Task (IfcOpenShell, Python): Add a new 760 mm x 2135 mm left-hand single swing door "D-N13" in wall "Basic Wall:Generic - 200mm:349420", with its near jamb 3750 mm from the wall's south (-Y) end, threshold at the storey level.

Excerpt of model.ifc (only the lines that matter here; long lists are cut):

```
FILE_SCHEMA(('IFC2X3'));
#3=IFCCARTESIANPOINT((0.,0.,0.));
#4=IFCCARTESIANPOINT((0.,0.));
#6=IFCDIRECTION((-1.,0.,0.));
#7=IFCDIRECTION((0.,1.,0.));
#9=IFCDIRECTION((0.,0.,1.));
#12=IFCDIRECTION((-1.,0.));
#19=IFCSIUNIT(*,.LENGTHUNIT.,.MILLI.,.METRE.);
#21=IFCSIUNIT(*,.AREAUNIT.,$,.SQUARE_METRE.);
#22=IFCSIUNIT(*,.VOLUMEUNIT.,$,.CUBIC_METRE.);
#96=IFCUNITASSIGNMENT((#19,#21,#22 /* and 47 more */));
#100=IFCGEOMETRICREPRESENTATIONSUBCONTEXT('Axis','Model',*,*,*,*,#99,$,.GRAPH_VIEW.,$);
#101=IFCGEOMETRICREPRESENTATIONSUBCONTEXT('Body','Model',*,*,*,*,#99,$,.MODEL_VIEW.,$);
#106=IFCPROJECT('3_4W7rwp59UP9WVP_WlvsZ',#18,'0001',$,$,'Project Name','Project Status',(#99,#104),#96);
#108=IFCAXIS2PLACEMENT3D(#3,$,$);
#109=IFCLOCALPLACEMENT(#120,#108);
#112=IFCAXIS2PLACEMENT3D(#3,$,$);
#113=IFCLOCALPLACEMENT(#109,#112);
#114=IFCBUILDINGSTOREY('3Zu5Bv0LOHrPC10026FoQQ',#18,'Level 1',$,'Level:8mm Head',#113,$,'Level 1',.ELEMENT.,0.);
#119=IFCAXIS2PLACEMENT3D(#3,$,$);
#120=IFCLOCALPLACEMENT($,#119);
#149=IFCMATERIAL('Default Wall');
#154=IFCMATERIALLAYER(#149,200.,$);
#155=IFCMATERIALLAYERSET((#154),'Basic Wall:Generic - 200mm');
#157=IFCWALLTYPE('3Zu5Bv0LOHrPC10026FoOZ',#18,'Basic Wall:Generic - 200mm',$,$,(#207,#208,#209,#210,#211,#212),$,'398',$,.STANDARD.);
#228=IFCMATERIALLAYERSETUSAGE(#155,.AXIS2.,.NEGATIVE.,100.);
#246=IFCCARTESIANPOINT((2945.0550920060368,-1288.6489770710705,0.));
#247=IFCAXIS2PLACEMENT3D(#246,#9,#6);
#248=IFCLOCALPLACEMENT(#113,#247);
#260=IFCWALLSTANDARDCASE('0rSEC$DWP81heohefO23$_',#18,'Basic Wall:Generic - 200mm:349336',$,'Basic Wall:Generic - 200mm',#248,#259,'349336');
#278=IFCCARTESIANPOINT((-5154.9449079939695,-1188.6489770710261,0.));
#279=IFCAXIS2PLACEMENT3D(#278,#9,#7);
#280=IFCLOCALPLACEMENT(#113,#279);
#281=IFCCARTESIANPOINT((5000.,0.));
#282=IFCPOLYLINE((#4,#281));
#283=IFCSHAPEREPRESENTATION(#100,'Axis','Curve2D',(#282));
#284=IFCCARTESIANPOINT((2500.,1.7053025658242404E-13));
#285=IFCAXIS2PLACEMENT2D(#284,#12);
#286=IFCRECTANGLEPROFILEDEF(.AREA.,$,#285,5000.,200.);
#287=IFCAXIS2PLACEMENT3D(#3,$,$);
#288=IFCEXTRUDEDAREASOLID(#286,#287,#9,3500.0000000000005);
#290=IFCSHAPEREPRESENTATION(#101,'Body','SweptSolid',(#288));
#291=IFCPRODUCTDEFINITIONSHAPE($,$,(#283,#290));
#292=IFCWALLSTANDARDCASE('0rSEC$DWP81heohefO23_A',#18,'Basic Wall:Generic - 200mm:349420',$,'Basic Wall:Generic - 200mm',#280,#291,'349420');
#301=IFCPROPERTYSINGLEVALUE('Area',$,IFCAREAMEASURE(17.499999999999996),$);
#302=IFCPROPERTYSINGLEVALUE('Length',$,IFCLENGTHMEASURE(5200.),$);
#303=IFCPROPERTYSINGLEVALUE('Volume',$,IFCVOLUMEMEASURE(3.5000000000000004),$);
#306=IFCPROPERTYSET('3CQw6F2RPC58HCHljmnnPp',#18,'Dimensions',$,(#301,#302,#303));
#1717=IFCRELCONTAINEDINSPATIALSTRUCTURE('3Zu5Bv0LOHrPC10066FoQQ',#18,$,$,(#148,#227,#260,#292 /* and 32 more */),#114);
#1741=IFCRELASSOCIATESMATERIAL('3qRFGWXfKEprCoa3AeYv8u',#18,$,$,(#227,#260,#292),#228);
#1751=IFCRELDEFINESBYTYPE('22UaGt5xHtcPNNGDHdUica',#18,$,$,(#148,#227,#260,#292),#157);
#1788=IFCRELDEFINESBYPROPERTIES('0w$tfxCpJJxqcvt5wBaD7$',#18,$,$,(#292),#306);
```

```python
import numpy as np
import ifcopenshell
import ifcopenshell.api.feature
import ifcopenshell.api.geometry
import ifcopenshell.api.pset
import ifcopenshell.api.root
import ifcopenshell.api.spatial
import ifcopenshell.api.type
import ifcopenshell.geom
import ifcopenshell.util.element
import ifcopenshell.util.placement
import ifcopenshell.util.representation
import ifcopenshell.util.shape
import ifcopenshell.util.unit

model = ifcopenshell.open("model.ifc")
unit_scale = ifcopenshell.util.unit.calculate_unit_scale(model)
area_scale = ifcopenshell.util.unit.calculate_unit_scale(model, "AREAUNIT")
volume_scale = ifcopenshell.util.unit.calculate_unit_scale(model, "VOLUMEUNIT")
settings = ifcopenshell.geom.settings()


def volume(element):
    """Net volume in cubic metres, openings subtracted."""
    shape = ifcopenshell.geom.create_shape(settings, element)
    return ifcopenshell.util.shape.get_volume(shape.geometry)


wall = model.by_guid("0rSEC$DWP81heohefO23_A")
storey = ifcopenshell.util.element.get_container(wall, ifc_class="IfcBuildingStorey")
context = ifcopenshell.util.representation.get_context(model, "Model", "Body", "MODEL_VIEW")
before = volume(wall)

width, height, from_end, sill = 0.76, 2.135, 3.75, 0.0  # metres

# The wall runs along its own X axis, and the end named is its -X end.
wall_shape = ifcopenshell.geom.create_shape(settings, wall)
x, y, z = ifcopenshell.util.shape.get_vertices(wall_shape.geometry).T
start = x.min() + from_end
face, thickness = float(y.min()), float(y.max() - y.min())
wall_matrix = ifcopenshell.util.placement.get_local_placement(wall.ObjectPlacement)
level = ifcopenshell.util.placement.get_local_placement(storey.ObjectPlacement)[2, 3]


def in_wall(x, y):
    """Placement at x, y metres in the wall's axes, at sill height."""
    matrix = wall_matrix.copy()
    matrix[:, 3] = wall_matrix @ np.array([x / unit_scale, y / unit_scale, 0.0, 1.0])
    matrix[2, 3] = level + sill / unit_scale
    return matrix


# Opening: a box that overshoots both wall faces by 50 mm.
opening = ifcopenshell.api.root.create_entity(model, ifc_class="IfcOpeningElement")
box = ifcopenshell.api.geometry.add_wall_representation(
    model, context=context, length=width, height=height, thickness=thickness + 0.1
)
ifcopenshell.api.geometry.assign_representation(model, product=opening, representation=box)
ifcopenshell.api.geometry.edit_object_placement(model, product=opening, matrix=in_wall(start, face - 0.05), is_si=False)
ifcopenshell.api.feature.add_feature(model, feature=opening, element=wall)

door = ifcopenshell.api.root.create_entity(model, ifc_class="IfcDoor", name="D-N13")
door.OverallWidth, door.OverallHeight = width / unit_scale, height / unit_scale
body = ifcopenshell.api.geometry.add_door_representation(
    model,
    context=context,
    overall_width=door.OverallWidth,
    overall_height=door.OverallHeight,
    operation_type="SINGLE_SWING_LEFT",
    lining_properties={"LiningDepth": thickness / unit_scale, "ThresholdDepth": thickness / unit_scale},
)
ifcopenshell.api.geometry.assign_representation(model, product=door, representation=body)
ifcopenshell.api.spatial.assign_container(model, products=[door], relating_structure=storey)
fills = ifcopenshell.api.feature.add_filling(model, opening=opening, element=door)
fills.OwnerHistory = door.OwnerHistory  # required in IFC2X3

# IFC2X3 keeps the operation on the door style.
style = ifcopenshell.api.root.create_entity(model, ifc_class="IfcDoorStyle", name="D-N13")
style.OperationType, style.ConstructionType = "SINGLE_SWING_LEFT", "NOTDEFINED"
style.ParameterTakesPrecedence = style.Sizeable = False
ifcopenshell.api.type.assign_type(model, related_objects=[door], relating_type=style)

# The lining spans the wall, so the door starts at the wall face.
ifcopenshell.api.geometry.edit_object_placement(model, product=door, matrix=in_wall(start, face), is_si=False)

after = volume(wall)

# Update the wall's stored quantities.
pset = model.by_id(ifcopenshell.util.element.get_pset(wall, "Dimensions", should_inherit=False)["id"])
ifcopenshell.api.pset.edit_pset(model, pset=pset, properties={
    "Area": model.create_entity("IfcAreaMeasure", after / thickness / area_scale),
    "Volume": model.create_entity("IfcVolumeMeasure", after / volume_scale),
})

print(f"wall volume {before:.3f} -> {after:.3f} m3")

model.write("model_rev.ifc")
```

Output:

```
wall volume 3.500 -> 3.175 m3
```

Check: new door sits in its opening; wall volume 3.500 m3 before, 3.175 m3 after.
